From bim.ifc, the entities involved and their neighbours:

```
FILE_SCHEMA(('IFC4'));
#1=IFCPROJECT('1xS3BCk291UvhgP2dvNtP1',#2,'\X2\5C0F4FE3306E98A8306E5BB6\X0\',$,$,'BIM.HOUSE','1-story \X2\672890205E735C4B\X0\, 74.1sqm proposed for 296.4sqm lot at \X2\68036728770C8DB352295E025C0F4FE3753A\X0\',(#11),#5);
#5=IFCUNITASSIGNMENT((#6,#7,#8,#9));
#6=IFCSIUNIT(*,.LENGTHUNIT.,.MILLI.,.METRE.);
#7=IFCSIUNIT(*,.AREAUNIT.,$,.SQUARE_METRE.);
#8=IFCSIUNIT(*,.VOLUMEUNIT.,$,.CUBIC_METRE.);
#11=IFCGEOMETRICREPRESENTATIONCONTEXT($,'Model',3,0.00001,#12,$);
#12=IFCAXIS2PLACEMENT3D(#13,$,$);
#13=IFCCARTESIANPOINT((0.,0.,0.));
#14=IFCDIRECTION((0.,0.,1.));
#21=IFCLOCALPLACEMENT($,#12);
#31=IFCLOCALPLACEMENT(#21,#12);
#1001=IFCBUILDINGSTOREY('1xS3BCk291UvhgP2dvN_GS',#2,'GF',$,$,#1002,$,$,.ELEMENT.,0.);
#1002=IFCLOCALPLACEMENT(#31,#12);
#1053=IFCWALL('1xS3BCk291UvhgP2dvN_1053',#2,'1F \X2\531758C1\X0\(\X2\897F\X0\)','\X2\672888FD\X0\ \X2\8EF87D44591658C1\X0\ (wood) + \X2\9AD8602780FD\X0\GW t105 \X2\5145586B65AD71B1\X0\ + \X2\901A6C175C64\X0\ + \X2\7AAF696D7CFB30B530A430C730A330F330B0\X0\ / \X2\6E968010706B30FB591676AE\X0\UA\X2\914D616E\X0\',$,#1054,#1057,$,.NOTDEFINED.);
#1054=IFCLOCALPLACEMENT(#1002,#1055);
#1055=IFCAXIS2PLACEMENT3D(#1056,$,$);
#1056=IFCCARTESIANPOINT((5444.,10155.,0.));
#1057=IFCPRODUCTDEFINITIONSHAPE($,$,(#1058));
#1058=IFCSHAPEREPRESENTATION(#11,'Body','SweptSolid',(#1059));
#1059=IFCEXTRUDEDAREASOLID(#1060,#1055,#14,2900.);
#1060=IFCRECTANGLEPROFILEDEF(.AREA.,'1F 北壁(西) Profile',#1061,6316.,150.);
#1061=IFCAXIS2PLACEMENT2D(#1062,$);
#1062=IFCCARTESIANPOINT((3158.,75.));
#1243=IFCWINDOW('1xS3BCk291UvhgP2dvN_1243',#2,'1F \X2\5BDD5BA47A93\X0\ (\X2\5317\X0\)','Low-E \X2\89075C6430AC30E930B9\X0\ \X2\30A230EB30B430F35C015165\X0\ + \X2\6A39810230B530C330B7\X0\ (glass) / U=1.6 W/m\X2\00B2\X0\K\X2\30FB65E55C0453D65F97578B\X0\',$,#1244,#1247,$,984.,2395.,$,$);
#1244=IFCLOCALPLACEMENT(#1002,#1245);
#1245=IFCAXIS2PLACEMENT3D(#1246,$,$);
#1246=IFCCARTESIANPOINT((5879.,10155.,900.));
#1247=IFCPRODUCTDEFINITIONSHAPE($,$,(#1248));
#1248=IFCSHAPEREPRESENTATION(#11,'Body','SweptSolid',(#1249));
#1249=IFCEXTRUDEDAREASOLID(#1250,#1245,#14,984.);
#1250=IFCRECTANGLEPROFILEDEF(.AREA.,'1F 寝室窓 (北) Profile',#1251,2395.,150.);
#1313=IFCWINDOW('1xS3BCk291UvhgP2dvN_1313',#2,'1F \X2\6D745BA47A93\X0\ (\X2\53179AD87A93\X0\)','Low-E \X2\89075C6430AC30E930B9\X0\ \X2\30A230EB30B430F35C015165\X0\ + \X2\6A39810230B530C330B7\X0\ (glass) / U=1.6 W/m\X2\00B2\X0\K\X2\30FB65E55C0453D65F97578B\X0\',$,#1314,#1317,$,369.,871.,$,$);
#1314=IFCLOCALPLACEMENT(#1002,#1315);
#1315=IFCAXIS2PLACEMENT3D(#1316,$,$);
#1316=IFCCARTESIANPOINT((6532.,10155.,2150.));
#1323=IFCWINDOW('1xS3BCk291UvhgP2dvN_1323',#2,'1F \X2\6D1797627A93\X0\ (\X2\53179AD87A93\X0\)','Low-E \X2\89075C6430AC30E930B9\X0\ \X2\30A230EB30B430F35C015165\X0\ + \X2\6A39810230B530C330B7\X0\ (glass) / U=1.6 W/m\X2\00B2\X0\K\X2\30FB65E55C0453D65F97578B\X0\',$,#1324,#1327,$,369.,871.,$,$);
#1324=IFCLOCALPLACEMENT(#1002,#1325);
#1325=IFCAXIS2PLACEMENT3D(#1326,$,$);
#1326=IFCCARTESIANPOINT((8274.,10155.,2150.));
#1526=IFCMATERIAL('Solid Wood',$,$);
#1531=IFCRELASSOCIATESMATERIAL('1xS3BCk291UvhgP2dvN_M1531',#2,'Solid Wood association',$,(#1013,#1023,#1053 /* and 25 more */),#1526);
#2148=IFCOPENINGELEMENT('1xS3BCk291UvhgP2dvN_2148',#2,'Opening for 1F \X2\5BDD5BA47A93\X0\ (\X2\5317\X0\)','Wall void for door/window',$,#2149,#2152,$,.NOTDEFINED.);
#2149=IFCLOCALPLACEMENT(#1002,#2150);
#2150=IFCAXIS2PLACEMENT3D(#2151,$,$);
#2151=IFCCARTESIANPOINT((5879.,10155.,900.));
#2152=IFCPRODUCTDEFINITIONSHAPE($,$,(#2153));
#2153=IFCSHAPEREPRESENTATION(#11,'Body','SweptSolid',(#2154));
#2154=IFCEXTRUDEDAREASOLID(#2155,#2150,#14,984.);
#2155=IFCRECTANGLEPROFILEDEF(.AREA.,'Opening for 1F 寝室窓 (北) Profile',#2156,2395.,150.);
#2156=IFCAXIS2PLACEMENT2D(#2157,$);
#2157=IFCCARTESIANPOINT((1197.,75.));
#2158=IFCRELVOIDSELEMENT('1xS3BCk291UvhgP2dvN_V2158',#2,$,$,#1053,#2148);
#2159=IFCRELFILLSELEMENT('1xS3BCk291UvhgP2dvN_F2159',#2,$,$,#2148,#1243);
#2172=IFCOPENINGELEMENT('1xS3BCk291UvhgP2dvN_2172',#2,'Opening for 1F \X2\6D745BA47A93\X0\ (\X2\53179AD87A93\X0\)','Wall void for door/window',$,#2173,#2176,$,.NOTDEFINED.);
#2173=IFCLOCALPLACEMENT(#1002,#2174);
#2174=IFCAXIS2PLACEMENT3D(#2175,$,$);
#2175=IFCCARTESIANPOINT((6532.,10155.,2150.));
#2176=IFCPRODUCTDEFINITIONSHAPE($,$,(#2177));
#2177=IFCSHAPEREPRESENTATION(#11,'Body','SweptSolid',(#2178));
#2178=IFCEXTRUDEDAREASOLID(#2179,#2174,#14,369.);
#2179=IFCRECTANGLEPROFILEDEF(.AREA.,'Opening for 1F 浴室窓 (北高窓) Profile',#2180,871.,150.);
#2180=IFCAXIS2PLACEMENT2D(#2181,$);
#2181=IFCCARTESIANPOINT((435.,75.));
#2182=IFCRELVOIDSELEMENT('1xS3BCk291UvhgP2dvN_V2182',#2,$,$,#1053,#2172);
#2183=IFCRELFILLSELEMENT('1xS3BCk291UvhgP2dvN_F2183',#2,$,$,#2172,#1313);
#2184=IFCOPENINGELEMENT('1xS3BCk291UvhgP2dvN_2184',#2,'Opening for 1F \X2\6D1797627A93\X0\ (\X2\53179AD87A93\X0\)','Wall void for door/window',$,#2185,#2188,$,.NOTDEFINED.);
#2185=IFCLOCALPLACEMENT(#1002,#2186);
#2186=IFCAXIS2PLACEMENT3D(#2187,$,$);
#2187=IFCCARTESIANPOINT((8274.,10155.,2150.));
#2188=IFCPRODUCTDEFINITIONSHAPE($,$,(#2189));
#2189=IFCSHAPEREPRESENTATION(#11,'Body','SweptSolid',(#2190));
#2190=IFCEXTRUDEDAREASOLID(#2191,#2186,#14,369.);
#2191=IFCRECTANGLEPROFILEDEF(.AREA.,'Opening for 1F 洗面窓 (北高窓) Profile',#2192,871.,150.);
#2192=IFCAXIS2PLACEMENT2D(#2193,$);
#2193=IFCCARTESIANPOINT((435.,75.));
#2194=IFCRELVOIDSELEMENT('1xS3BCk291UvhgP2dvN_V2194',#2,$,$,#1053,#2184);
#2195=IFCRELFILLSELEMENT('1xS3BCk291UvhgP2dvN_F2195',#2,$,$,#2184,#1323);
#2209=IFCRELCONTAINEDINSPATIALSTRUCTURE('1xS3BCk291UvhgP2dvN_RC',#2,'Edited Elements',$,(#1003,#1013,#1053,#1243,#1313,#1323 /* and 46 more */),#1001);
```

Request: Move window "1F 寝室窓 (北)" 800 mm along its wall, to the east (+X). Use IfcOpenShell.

```python
import ifcopenshell
import ifcopenshell.api.geometry
import ifcopenshell.util.placement
import ifcopenshell.util.unit

model = ifcopenshell.open("bim.ifc")
unit_scale = ifcopenshell.util.unit.calculate_unit_scale(model)

window = model.by_id(1243)
opening = window.FillsVoids[0].RelatingOpeningElement
wall = opening.VoidsElements[0].RelatingBuildingElement

wall_matrix = ifcopenshell.util.placement.get_local_placement(wall.ObjectPlacement)
shift = wall_matrix[:3, 0] * 0.8 / unit_scale
before = ifcopenshell.util.placement.get_local_placement(window.ObjectPlacement)[:3, 3].copy()

# The window is not placed relative to its opening, so move both.
for product in (opening, window):
    matrix = ifcopenshell.util.placement.get_local_placement(product.ObjectPlacement)
    matrix[:3, 3] += shift
    ifcopenshell.api.geometry.edit_object_placement(model, product=product, matrix=matrix, is_si=False)

after = ifcopenshell.util.placement.get_local_placement(window.ObjectPlacement)[:3, 3]
print("window moved by", (after - before).round(3) + 0.0)

model.write("bim-out.ifc")
```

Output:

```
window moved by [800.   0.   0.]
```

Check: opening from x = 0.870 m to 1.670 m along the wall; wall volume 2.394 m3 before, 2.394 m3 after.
